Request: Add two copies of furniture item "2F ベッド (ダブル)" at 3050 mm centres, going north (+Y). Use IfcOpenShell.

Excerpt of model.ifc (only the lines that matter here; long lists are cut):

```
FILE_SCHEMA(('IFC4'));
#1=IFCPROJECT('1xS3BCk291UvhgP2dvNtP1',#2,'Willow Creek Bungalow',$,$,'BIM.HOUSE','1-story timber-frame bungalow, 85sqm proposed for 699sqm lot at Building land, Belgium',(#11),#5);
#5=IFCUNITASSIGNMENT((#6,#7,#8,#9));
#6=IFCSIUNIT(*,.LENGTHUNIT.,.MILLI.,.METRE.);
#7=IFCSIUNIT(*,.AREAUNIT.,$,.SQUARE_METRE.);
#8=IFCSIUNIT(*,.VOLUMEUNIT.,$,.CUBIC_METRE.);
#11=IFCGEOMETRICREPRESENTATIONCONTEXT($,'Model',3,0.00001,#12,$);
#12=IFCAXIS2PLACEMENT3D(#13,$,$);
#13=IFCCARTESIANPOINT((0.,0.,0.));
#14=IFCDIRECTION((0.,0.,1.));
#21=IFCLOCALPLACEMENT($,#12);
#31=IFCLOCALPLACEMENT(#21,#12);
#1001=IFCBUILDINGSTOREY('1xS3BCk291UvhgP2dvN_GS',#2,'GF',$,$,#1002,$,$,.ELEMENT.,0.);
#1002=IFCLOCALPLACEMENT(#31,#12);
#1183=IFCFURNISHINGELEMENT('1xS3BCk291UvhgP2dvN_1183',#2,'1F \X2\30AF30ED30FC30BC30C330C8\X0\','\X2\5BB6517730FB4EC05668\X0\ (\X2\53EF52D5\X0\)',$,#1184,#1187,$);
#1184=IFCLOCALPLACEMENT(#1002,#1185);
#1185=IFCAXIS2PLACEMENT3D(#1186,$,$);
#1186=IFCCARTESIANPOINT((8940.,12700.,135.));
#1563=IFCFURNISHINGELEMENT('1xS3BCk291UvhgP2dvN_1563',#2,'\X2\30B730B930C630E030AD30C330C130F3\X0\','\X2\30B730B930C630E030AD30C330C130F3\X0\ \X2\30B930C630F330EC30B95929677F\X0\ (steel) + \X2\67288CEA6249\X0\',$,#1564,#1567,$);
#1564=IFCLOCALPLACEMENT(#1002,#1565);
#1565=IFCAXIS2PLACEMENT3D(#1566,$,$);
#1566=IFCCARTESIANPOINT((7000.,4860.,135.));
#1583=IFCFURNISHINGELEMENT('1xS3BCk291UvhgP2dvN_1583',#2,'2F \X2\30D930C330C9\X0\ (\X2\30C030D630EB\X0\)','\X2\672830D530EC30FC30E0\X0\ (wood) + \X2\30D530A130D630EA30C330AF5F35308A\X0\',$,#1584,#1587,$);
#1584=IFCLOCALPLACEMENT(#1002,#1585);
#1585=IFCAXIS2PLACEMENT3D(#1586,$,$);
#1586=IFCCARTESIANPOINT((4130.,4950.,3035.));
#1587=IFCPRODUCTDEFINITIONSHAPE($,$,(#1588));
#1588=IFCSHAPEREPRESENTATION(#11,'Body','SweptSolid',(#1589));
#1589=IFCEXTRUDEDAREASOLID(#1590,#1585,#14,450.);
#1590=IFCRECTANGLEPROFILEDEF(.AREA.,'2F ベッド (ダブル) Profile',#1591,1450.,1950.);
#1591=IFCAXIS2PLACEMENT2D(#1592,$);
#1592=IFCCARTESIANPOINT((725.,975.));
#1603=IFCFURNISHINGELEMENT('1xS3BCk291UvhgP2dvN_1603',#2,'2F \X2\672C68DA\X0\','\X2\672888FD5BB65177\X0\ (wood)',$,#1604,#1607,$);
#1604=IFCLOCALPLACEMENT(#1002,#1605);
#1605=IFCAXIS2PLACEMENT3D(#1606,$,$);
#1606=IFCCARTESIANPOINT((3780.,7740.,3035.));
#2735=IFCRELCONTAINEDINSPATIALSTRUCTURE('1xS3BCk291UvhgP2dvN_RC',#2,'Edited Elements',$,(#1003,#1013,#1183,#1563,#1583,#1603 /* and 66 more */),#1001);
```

```python
import numpy as np
import ifcopenshell
import ifcopenshell.api.geometry
import ifcopenshell.api.root
import ifcopenshell.util.element
import ifcopenshell.util.placement
import ifcopenshell.util.unit

model = ifcopenshell.open("model.ifc")
unit_scale = ifcopenshell.util.unit.calculate_unit_scale(model)


def reuse_history(source, copy):
    """copy_class also copies each property set's owner history, people and application; keep the originals."""
    for rel in copy.IsDefinedBy:
        if rel.is_a("IfcRelDefinesByProperties") and (history := rel.RelatingPropertyDefinition.OwnerHistory):
            rel.RelatingPropertyDefinition.OwnerHistory = source.OwnerHistory
            ifcopenshell.util.element.remove_deep2(model, history)


source = model.by_guid("1xS3BCk291UvhgP2dvN_1583")
base = ifcopenshell.util.placement.get_local_placement(source.ObjectPlacement)
step = np.array([0.0, 1.0, 0.0]) * 3.05 / unit_scale

for i in range(1, 3):
    copy = ifcopenshell.api.root.copy_class(model, product=source)
    copy.Representation = ifcopenshell.util.element.copy_deep(
        model, source.Representation, exclude=["IfcGeometricRepresentationContext", "IfcRepresentationMap"]
    )
    reuse_history(source, copy)
    matrix = base.copy()
    matrix[:3, 3] += i * step
    print("added at", matrix[:3, 3].round(3) + 0.0)
    ifcopenshell.api.geometry.edit_object_placement(model, product=copy, matrix=matrix, is_si=False)

model.write("model_rev.ifc")
```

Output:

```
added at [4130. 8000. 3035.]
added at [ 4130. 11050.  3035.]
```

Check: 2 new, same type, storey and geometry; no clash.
